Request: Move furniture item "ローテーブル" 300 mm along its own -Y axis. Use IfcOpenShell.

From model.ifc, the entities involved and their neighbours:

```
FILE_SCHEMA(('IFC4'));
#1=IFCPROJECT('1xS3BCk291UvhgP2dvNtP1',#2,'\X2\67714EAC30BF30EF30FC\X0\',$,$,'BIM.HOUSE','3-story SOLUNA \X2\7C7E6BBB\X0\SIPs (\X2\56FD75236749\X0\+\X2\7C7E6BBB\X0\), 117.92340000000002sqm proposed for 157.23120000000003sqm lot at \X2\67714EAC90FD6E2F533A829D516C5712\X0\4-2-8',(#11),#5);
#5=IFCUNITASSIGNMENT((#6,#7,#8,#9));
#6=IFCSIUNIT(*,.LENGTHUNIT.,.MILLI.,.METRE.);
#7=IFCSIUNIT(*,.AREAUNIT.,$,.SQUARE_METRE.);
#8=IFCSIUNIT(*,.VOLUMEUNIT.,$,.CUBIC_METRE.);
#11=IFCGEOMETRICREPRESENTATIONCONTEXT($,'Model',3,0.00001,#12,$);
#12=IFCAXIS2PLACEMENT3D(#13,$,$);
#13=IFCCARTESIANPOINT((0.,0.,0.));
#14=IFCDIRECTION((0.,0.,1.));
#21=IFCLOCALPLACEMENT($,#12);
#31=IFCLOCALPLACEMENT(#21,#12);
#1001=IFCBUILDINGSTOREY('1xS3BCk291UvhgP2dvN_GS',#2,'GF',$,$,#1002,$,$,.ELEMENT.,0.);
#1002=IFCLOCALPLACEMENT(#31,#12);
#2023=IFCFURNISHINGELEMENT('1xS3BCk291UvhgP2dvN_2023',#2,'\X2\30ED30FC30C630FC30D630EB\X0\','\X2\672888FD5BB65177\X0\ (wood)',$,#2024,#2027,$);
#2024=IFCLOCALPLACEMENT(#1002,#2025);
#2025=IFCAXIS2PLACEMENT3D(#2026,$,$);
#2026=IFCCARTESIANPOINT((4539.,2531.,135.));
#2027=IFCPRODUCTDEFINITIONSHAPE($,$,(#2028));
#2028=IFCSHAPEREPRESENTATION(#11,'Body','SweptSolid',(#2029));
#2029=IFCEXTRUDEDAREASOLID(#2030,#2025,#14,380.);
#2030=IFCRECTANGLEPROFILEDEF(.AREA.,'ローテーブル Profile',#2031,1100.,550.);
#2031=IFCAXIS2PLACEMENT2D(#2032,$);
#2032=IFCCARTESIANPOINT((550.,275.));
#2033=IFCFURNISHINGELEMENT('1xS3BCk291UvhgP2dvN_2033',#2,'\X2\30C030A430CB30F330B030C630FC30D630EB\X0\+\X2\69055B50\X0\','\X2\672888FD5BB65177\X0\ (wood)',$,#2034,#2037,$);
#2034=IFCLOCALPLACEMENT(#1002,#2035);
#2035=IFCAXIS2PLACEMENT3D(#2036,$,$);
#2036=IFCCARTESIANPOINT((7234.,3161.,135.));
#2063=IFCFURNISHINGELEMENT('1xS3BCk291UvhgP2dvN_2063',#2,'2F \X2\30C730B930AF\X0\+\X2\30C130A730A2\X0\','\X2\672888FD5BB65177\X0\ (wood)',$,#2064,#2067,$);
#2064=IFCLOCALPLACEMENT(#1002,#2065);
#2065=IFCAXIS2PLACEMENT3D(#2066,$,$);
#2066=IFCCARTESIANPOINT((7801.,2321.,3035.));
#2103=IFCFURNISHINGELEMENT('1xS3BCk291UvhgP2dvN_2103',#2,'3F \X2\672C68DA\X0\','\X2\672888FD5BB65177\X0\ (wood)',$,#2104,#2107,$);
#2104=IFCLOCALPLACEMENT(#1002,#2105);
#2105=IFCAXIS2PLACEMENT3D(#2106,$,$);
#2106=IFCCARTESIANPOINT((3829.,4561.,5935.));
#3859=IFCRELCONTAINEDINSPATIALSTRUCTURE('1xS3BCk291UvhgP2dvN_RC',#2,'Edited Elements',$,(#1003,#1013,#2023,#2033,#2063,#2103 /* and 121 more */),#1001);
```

```python
import ifcopenshell
import ifcopenshell.api.geometry
import ifcopenshell.util.placement
import ifcopenshell.util.unit

model = ifcopenshell.open("model.ifc")
unit_scale = ifcopenshell.util.unit.calculate_unit_scale(model)

item = model.by_guid("1xS3BCk291UvhgP2dvN_2023")
matrix = ifcopenshell.util.placement.get_local_placement(item.ObjectPlacement)
matrix[:3, 3] -= matrix[:3, 1] * 0.3 / unit_scale
ifcopenshell.api.geometry.edit_object_placement(model, product=item, matrix=matrix, is_si=False)

print(ifcopenshell.util.placement.get_local_placement(item.ObjectPlacement).round(3) + 0.0)

model.write("model_edited.ifc")
```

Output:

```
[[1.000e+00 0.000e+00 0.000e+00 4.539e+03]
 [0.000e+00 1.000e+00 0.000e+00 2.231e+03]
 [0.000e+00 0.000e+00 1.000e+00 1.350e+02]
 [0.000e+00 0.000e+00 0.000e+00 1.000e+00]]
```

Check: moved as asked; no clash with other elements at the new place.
